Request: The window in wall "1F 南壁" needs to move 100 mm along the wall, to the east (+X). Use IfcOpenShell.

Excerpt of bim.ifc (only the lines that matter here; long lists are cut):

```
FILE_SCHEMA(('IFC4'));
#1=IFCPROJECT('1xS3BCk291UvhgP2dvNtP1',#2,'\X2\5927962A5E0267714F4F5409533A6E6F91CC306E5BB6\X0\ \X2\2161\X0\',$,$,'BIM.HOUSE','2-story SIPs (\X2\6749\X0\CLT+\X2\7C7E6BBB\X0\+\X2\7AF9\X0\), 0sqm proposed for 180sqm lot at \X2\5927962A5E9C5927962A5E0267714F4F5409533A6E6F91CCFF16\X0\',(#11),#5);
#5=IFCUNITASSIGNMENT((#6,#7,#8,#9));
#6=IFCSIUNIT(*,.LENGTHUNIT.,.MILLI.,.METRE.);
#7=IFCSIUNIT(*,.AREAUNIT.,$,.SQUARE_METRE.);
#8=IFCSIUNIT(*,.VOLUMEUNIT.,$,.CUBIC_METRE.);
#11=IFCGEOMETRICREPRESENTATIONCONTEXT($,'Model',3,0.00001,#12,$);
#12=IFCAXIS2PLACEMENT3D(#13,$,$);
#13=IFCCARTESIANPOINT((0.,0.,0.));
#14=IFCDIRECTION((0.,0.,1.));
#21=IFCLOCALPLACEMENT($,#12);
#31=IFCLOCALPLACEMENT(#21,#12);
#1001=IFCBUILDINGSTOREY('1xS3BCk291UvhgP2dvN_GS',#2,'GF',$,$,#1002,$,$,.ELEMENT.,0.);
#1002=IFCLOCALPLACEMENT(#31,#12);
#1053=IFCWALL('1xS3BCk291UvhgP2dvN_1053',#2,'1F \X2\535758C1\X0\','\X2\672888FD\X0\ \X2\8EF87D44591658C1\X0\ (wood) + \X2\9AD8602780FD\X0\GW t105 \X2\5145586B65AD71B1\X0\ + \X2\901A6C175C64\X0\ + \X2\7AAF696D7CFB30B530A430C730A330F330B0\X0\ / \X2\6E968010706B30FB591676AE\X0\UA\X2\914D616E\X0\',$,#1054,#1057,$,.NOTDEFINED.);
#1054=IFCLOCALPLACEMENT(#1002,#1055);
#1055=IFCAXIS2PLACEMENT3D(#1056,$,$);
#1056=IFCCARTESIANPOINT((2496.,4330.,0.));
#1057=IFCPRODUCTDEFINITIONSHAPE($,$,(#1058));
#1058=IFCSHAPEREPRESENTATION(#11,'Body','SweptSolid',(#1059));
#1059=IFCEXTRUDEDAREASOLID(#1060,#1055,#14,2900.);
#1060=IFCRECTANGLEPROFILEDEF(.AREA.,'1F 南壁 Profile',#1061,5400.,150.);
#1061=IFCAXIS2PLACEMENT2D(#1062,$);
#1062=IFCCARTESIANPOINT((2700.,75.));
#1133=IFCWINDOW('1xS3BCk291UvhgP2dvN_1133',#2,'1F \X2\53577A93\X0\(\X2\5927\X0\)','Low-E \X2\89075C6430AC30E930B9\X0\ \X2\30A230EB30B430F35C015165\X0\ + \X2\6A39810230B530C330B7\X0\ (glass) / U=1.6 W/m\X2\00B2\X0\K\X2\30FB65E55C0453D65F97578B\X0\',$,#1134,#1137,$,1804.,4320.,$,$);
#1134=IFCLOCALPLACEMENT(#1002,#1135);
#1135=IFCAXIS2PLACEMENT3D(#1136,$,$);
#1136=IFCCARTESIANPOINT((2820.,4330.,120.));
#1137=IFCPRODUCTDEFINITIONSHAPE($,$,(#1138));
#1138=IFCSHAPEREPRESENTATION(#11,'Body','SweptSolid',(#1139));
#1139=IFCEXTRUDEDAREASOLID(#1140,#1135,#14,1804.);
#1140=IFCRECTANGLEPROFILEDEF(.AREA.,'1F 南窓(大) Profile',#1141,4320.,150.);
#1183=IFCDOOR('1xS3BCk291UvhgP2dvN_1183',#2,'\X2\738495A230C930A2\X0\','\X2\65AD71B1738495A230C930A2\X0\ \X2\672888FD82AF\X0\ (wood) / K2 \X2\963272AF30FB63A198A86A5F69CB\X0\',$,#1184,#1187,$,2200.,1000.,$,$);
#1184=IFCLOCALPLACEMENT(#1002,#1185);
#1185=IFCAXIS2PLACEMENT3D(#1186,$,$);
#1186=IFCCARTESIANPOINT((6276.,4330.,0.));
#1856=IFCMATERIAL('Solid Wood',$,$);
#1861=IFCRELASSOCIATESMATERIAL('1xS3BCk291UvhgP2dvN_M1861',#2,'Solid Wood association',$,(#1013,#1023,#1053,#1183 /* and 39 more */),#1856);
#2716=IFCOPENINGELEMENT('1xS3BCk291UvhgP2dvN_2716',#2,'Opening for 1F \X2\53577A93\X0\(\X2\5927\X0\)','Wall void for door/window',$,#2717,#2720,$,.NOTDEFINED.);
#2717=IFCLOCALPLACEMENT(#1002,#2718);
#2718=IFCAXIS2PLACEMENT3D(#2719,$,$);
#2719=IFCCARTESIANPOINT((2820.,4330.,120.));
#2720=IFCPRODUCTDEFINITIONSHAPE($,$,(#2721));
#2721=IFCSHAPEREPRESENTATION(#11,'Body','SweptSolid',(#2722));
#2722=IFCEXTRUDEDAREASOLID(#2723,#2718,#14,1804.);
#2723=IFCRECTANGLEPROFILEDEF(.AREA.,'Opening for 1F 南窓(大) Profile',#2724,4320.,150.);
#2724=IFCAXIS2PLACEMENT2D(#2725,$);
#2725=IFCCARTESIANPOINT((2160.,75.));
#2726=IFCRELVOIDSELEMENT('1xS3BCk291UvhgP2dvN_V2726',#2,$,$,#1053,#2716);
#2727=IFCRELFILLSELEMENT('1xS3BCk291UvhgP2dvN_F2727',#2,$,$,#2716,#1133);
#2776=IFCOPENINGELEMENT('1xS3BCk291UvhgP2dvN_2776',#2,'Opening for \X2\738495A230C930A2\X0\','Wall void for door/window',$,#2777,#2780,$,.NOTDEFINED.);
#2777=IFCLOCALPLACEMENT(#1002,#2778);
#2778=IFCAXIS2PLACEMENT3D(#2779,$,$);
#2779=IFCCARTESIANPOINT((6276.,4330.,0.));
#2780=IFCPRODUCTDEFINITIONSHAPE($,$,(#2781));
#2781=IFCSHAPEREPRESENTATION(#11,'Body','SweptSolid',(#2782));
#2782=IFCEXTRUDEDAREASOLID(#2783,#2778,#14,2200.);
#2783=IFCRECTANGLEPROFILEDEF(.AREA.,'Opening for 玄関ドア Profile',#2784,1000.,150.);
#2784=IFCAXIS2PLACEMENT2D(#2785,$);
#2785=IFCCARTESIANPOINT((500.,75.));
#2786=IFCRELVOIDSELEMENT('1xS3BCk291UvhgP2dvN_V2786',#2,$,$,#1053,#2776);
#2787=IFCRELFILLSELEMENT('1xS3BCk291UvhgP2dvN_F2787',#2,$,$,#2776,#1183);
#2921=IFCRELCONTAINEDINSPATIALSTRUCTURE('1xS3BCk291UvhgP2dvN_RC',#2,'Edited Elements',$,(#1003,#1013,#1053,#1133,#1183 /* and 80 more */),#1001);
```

```python
import ifcopenshell
import ifcopenshell.api.geometry
import ifcopenshell.util.placement
import ifcopenshell.util.unit

model = ifcopenshell.open("bim.ifc")
unit_scale = ifcopenshell.util.unit.calculate_unit_scale(model)

window = model.by_guid("1xS3BCk291UvhgP2dvN_1133")
opening = window.FillsVoids[0].RelatingOpeningElement
wall = opening.VoidsElements[0].RelatingBuildingElement

wall_matrix = ifcopenshell.util.placement.get_local_placement(wall.ObjectPlacement)
shift = wall_matrix[:3, 0] * 0.1 / unit_scale
before = ifcopenshell.util.placement.get_local_placement(window.ObjectPlacement)[:3, 3].copy()

# The window is not placed relative to its opening, so move both.
for product in (opening, window):
    matrix = ifcopenshell.util.placement.get_local_placement(product.ObjectPlacement)
    matrix[:3, 3] += shift
    ifcopenshell.api.geometry.edit_object_placement(model, product=product, matrix=matrix, is_si=False)

after = ifcopenshell.util.placement.get_local_placement(window.ObjectPlacement)[:3, 3]
print("window moved by", (after - before).round(3) + 0.0)

model.write("bim_edited.ifc")
```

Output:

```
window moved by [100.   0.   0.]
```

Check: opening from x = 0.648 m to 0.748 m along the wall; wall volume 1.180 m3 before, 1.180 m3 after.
